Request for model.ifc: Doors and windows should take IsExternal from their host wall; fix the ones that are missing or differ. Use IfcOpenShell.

First a look at what the model holds.

```python
import ifcopenshell
import ifcopenshell.util.element

model = ifcopenshell.open("model.ifc")
print(model.schema)
seen = {}
for e in model.by_type("IfcDoor") + model.by_type("IfcWindow"):
    if not e.FillsVoids:
        continue
    host = e.FillsVoids[0].RelatingOpeningElement.VoidsElements[0].RelatingBuildingElement
    own = ifcopenshell.util.element.get_pset(e, f"Pset_{e.is_a()[3:].removesuffix('StandardCase')}Common", "IsExternal")
    wall = ifcopenshell.util.element.get_pset(host, "Pset_WallCommon", "IsExternal")
    seen[e.is_a(), own, wall] = seen.get((e.is_a(), own, wall), 0) + 1
for (cls, own, wall), count in sorted(seen.items(), key=str):
    print(count, cls, "IsExternal:", own, "| host wall:", wall)
```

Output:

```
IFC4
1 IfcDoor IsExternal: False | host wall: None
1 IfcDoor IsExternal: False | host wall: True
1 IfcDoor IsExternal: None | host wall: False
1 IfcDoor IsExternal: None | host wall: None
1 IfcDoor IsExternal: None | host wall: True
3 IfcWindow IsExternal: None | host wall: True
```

```python
import ifcopenshell
import ifcopenshell.api.pset
import ifcopenshell.util.element

model = ifcopenshell.open("model.ifc")

count = 0
for ifc_class, pset_name in (("IfcDoor", "Pset_DoorCommon"), ("IfcWindow", "Pset_WindowCommon")):
    for e in model.by_type(ifc_class):
        if not e.FillsVoids:
            continue
        host = e.FillsVoids[0].RelatingOpeningElement.VoidsElements[0].RelatingBuildingElement
        external = ifcopenshell.util.element.get_pset(host, "Pset_WallCommon", "IsExternal")
        if external is None or ifcopenshell.util.element.get_pset(e, pset_name, "IsExternal") == external:
            continue
        pset = ifcopenshell.api.pset.add_pset(model, product=e, name=pset_name)
        ifcopenshell.api.pset.edit_pset(model, pset=pset, properties={"IsExternal": external})
        count += 1

print(count, "updated")

model.write("model_edited.ifc")
```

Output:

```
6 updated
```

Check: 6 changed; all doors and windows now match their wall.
